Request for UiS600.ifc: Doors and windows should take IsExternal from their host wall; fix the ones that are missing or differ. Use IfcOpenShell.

First a look at what the model holds.

```python
import ifcopenshell
import ifcopenshell.util.element

model = ifcopenshell.open("UiS600.ifc")
print(model.schema)
seen = {}
for e in model.by_type("IfcDoor") + model.by_type("IfcWindow"):
    if not e.FillsVoids:
        continue
    host = e.FillsVoids[0].RelatingOpeningElement.VoidsElements[0].RelatingBuildingElement
    own = ifcopenshell.util.element.get_pset(e, f"Pset_{e.is_a()[3:].removesuffix('StandardCase')}Common", "IsExternal")
    wall = ifcopenshell.util.element.get_pset(host, "Pset_WallCommon", "IsExternal")
    seen[e.is_a(), own, wall] = seen.get((e.is_a(), own, wall), 0) + 1
for (cls, own, wall), count in sorted(seen.items(), key=str):
    print(count, cls, "IsExternal:", own, "| host wall:", wall)
```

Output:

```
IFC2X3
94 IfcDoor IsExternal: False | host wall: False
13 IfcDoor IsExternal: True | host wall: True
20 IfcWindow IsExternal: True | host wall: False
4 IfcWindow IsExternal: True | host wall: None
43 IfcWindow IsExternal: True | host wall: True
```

```python
import ifcopenshell
import ifcopenshell.api.pset
import ifcopenshell.util.element

model = ifcopenshell.open("UiS600.ifc")

count = 0
for ifc_class, pset_name in (("IfcDoor", "Pset_DoorCommon"), ("IfcWindow", "Pset_WindowCommon")):
    for e in model.by_type(ifc_class):
        if not e.FillsVoids:
            continue
        host = e.FillsVoids[0].RelatingOpeningElement.VoidsElements[0].RelatingBuildingElement
        external = ifcopenshell.util.element.get_pset(host, "Pset_WallCommon", "IsExternal")
        if external is None or ifcopenshell.util.element.get_pset(e, pset_name, "IsExternal") == external:
            continue
        found = ifcopenshell.util.element.get_pset(e, pset_name, should_inherit=False)
        if found:
            pset = model.by_id(found["id"])
            if len(ifcopenshell.util.element.get_elements_by_pset(pset)) > 1:
                pset = ifcopenshell.api.pset.unshare_pset(model, products=[e], pset=pset)[0]
        else:
            pset = ifcopenshell.api.pset.add_pset(model, product=e, name=pset_name)
        ifcopenshell.api.pset.edit_pset(model, pset=pset, properties={"IsExternal": external})
        count += 1

print(count, "updated")

model.write("UiS600_edited.ifc")
```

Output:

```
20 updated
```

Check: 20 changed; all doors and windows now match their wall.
